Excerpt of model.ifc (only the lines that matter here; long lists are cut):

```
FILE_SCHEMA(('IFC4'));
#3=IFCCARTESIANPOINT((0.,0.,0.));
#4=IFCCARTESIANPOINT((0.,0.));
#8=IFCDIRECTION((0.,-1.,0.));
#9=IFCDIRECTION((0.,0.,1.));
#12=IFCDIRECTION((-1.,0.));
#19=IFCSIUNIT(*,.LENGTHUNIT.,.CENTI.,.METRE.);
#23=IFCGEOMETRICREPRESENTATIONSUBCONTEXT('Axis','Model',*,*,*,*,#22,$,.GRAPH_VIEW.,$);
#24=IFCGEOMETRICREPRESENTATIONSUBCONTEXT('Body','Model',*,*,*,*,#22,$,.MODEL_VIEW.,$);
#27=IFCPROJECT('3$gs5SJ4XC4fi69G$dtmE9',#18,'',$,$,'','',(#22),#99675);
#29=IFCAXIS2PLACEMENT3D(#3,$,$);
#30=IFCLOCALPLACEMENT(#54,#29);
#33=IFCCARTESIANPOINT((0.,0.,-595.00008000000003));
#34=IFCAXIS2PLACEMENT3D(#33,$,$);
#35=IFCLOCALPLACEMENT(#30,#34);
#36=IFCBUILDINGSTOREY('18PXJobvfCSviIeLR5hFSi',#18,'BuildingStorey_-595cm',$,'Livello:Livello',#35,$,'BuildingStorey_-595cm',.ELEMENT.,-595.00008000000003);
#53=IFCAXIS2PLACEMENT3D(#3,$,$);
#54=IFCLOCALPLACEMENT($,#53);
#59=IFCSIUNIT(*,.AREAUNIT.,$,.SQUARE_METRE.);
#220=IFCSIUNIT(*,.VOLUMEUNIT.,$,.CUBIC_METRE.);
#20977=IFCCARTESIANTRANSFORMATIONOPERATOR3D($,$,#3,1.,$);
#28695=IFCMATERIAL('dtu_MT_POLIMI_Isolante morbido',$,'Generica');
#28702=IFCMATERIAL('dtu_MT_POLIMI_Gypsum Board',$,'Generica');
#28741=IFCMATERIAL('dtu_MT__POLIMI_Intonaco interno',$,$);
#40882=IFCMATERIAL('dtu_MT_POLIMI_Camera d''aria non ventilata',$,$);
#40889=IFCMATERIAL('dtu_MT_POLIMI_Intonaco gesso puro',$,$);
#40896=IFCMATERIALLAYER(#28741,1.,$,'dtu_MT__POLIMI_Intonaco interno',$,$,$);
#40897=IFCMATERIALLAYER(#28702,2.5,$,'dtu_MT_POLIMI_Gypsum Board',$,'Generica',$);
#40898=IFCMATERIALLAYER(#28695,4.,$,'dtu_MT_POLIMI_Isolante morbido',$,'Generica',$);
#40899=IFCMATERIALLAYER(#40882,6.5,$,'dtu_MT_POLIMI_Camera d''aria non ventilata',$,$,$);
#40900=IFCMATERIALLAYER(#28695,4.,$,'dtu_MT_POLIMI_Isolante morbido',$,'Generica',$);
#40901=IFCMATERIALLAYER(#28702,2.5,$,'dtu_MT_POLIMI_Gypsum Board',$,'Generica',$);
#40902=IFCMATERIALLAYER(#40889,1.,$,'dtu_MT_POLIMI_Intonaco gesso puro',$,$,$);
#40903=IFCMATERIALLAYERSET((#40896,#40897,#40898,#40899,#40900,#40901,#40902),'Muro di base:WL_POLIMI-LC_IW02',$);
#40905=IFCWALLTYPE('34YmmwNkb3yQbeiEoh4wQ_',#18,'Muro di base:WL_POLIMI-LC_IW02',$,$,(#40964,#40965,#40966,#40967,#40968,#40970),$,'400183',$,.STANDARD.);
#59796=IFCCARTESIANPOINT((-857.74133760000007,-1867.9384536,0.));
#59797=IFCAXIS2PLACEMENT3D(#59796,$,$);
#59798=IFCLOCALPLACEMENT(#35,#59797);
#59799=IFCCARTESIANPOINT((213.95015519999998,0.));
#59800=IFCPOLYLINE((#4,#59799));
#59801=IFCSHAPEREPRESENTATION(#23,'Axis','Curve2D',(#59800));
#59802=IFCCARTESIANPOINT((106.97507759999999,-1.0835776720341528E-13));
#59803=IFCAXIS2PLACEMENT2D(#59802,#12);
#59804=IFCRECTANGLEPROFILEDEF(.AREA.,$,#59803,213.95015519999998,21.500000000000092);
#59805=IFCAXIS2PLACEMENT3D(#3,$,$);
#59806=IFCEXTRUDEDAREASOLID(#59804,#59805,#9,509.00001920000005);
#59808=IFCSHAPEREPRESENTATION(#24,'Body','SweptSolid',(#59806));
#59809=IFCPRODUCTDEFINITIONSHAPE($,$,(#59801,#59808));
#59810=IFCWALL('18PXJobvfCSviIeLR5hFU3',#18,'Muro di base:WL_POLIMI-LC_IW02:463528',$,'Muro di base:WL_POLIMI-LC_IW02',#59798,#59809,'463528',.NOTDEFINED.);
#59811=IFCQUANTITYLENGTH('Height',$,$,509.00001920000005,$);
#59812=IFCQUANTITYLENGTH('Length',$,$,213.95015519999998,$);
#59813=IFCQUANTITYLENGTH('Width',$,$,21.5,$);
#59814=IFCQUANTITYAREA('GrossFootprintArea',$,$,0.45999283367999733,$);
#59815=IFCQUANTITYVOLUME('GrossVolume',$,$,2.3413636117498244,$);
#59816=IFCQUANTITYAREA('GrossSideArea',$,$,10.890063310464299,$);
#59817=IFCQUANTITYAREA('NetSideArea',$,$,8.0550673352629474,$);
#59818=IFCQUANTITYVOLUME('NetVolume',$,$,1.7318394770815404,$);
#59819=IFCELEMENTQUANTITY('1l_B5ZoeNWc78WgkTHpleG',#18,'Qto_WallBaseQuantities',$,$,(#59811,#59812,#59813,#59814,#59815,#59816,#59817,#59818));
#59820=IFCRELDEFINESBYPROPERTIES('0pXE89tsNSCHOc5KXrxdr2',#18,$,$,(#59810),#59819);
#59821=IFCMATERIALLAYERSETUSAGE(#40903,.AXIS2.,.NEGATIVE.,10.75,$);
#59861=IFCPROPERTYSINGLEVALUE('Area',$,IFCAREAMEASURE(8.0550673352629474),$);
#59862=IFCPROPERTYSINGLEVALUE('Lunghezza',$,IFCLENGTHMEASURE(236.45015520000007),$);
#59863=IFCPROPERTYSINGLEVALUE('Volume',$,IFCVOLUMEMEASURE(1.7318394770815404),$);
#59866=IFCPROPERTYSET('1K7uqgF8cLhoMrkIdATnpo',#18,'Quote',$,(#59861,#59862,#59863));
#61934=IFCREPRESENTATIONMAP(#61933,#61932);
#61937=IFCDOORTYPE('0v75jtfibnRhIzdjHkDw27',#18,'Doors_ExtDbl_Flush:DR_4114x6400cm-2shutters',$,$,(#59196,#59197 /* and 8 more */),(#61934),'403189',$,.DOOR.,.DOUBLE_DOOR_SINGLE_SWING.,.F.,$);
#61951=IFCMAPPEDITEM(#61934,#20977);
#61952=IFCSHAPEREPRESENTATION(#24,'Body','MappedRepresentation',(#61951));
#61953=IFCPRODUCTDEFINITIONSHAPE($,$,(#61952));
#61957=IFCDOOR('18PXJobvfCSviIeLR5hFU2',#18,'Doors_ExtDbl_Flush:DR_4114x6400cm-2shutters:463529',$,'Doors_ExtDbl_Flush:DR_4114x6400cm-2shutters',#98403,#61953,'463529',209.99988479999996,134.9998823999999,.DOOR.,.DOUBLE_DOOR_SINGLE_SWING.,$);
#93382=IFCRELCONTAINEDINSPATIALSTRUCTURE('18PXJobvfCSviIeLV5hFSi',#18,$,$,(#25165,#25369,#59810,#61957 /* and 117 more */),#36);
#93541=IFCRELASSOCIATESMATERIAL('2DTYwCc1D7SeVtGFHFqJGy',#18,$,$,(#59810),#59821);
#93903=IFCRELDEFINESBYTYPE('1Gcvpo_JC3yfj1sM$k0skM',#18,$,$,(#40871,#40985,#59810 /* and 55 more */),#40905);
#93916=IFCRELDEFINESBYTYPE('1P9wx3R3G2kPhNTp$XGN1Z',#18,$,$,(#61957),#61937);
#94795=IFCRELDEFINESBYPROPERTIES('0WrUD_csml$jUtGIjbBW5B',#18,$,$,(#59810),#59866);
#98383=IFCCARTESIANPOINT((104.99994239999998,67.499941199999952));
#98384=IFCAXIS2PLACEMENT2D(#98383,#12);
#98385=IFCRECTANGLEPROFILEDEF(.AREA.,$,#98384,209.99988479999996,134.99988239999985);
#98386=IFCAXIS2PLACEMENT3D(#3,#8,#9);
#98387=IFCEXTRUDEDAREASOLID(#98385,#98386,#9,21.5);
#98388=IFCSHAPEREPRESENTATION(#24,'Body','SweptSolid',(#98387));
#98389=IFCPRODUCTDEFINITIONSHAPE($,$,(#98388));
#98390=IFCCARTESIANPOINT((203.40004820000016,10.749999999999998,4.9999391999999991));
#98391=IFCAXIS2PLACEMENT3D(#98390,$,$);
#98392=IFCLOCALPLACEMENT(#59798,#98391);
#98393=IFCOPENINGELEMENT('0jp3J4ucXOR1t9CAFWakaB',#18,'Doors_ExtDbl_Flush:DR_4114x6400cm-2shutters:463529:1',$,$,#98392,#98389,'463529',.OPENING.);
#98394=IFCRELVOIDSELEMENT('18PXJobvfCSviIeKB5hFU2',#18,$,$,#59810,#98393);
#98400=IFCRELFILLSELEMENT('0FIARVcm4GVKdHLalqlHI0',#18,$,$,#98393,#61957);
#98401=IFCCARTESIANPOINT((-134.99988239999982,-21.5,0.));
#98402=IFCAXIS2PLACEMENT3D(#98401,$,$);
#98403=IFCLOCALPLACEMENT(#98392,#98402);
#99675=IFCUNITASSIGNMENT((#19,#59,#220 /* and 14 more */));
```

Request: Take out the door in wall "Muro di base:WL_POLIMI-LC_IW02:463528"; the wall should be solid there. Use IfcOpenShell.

```python
import ifcopenshell
import ifcopenshell.api.feature
import ifcopenshell.api.pset
import ifcopenshell.api.root
import ifcopenshell.geom
import ifcopenshell.util.element
import ifcopenshell.util.shape
import ifcopenshell.util.unit

model = ifcopenshell.open("model.ifc")
area_scale = ifcopenshell.util.unit.calculate_unit_scale(model, "AREAUNIT")
volume_scale = ifcopenshell.util.unit.calculate_unit_scale(model, "VOLUMEUNIT")
settings = ifcopenshell.geom.settings()


def volume(element):
    """Net volume in cubic metres, openings subtracted."""
    shape = ifcopenshell.geom.create_shape(settings, element)
    return ifcopenshell.util.shape.get_volume(shape.geometry)


door = model.by_guid("18PXJobvfCSviIeLR5hFU2")
opening = door.FillsVoids[0].RelatingOpeningElement
wall = opening.VoidsElements[0].RelatingBuildingElement
before = volume(wall)

ifcopenshell.api.root.remove_product(model, product=door)
ifcopenshell.api.feature.remove_feature(model, feature=opening)

after = volume(wall)
thickness = 0.215  # wall thickness in metres

# Update the wall's stored quantities.
qto = model.by_id(ifcopenshell.util.element.get_pset(wall, "Qto_WallBaseQuantities", should_inherit=False)["id"])
ifcopenshell.api.pset.edit_qto(model, qto=qto, properties={
    "NetSideArea": after / thickness / area_scale,
    "NetVolume": after / volume_scale,
})
pset = model.by_id(ifcopenshell.util.element.get_pset(wall, "Quote", should_inherit=False)["id"])
ifcopenshell.api.pset.edit_pset(model, pset=pset, properties={
    "Area": model.create_entity("IfcAreaMeasure", after / thickness / area_scale),
    "Volume": model.create_entity("IfcVolumeMeasure", after / volume_scale),
})

print(f"wall volume {before:.3f} -> {after:.3f} m3")

model.write("model_edited.ifc")
```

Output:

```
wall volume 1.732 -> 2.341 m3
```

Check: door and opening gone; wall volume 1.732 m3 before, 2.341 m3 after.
